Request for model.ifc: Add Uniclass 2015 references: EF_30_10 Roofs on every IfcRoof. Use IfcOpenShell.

First a look at what the model holds.

```python
import ifcopenshell

model = ifcopenshell.open("model.ifc")
print(model.schema)
print("classifications:", [c.Name for c in model.by_type("IfcClassification")])
for ifc_class in ("IfcDoor", "IfcRoof", "IfcStair", "IfcWall", "IfcWindow"):
    print(ifc_class, len(model.by_type(ifc_class)))
```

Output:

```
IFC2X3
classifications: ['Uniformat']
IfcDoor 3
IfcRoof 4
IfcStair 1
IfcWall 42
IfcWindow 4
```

```python
import ifcopenshell
import ifcopenshell.api.classification

model = ifcopenshell.open("model.ifc")

# IFC2X3 requires Source and Edition and has no link from the project to the system.
system = model.create_entity("IfcClassification", Source="NBS", Edition="2015", Name="Uniclass 2015")

codes = {
    "IfcRoof": ("EF_30_10", "Roofs"),
}
for ifc_class, (code, name) in codes.items():
    products = model.by_type(ifc_class)
    ifcopenshell.api.classification.add_reference(
        model, products=products, classification=system, identification=code, name=name
    )
    print(code, len(products))

model.write("model_rev.ifc")
```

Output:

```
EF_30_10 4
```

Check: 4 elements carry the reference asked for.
